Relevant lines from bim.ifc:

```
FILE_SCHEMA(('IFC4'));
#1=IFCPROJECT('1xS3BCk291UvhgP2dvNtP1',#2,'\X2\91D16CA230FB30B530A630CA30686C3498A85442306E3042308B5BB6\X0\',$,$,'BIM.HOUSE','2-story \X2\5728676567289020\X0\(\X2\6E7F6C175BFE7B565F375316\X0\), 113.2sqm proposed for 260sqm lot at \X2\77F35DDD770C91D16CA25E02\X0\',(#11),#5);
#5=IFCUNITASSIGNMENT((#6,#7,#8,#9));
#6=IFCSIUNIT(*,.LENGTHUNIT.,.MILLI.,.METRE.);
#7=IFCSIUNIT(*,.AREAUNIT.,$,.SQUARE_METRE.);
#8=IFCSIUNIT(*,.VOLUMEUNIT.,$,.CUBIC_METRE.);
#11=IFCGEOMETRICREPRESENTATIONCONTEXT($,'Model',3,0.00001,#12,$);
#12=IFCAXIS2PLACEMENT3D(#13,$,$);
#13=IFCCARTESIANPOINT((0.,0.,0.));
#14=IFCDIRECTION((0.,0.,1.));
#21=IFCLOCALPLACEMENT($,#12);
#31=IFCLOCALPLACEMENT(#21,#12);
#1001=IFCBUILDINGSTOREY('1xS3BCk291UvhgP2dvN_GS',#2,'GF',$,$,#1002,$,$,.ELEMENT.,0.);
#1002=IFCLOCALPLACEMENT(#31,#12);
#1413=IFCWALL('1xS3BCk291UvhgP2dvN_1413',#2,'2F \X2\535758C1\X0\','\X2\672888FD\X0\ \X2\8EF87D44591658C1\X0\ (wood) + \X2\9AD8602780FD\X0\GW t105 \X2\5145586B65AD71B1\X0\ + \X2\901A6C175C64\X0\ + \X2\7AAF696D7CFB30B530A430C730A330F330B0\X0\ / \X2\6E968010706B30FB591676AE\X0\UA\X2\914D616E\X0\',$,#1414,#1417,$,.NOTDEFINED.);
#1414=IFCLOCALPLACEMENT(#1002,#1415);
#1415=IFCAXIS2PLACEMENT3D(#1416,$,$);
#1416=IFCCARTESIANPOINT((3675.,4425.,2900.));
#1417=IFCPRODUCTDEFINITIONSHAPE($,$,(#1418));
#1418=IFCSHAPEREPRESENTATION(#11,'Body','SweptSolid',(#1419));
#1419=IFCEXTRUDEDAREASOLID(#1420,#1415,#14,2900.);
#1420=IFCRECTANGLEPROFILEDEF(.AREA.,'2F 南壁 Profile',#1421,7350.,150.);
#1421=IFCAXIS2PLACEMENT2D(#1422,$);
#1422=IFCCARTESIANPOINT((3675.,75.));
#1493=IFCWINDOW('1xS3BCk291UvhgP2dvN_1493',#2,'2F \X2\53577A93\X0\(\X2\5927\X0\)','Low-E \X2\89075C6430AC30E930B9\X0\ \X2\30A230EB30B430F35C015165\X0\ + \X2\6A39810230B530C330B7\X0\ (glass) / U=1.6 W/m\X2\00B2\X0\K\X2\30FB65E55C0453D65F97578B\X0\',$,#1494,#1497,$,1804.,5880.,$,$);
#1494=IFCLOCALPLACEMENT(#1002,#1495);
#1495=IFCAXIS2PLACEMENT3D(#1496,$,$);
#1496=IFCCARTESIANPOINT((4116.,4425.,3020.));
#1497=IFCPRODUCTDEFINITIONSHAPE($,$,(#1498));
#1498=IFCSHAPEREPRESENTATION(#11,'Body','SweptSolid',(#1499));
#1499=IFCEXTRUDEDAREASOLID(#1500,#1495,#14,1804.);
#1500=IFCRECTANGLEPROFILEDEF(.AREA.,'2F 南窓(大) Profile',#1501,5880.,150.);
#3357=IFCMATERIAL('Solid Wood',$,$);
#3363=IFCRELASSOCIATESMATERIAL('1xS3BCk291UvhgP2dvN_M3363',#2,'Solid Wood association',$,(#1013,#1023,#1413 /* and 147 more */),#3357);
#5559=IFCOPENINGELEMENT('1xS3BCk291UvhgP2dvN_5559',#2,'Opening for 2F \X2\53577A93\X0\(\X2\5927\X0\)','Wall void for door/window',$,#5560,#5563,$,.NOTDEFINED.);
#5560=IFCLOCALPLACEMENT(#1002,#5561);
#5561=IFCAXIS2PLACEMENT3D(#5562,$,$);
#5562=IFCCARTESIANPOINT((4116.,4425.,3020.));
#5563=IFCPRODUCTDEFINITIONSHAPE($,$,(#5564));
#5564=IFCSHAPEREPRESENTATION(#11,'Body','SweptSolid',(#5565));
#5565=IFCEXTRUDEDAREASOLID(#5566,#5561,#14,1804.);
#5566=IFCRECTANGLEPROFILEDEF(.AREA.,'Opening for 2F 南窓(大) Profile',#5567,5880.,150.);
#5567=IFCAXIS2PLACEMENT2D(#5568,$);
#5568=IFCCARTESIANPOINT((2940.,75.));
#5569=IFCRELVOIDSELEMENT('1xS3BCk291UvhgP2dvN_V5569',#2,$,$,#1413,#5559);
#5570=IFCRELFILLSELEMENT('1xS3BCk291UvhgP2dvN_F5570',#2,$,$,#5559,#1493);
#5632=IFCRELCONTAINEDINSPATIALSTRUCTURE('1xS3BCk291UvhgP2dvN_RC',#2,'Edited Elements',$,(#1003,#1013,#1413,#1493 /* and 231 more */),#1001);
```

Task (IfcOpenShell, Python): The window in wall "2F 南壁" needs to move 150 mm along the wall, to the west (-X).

```python
import ifcopenshell
import ifcopenshell.api.geometry
import ifcopenshell.util.placement
import ifcopenshell.util.unit

model = ifcopenshell.open("bim.ifc")
unit_scale = ifcopenshell.util.unit.calculate_unit_scale(model)

window = model.by_id(1493)
opening = window.FillsVoids[0].RelatingOpeningElement
wall = opening.VoidsElements[0].RelatingBuildingElement

wall_matrix = ifcopenshell.util.placement.get_local_placement(wall.ObjectPlacement)
shift = wall_matrix[:3, 0] * -0.15 / unit_scale
before = ifcopenshell.util.placement.get_local_placement(window.ObjectPlacement)[:3, 3].copy()

# The window is not placed relative to its opening, so move both.
for product in (opening, window):
    matrix = ifcopenshell.util.placement.get_local_placement(product.ObjectPlacement)
    matrix[:3, 3] += shift
    ifcopenshell.api.geometry.edit_object_placement(model, product=product, matrix=matrix, is_si=False)

after = ifcopenshell.util.placement.get_local_placement(window.ObjectPlacement)[:3, 3]
print("window moved by", (after - before).round(3) + 0.0)

model.write("bim_rev.ifc")
```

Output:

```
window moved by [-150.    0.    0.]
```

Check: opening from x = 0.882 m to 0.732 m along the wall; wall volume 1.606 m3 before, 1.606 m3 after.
